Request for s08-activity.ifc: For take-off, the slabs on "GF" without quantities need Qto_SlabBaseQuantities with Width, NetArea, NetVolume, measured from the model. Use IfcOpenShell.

First a look at what the model holds.

```python
import ifcopenshell
import ifcopenshell.util.element
import ifcopenshell.util.unit

model = ifcopenshell.open("s08-activity.ifc")
print(model.schema)
for unit_type in ("LENGTHUNIT", "AREAUNIT", "VOLUMEUNIT"):
    print(unit_type, ifcopenshell.util.unit.calculate_unit_scale(model, unit_type))
storey = next(s for s in model.by_type("IfcBuildingStorey") if s.Name == "GF")
slabs = [e for e in ifcopenshell.util.element.get_decomposition(storey) if e.is_a("IfcSlab")]
for e in sorted(slabs, key=lambda e: e.id()):
    print(e.id(), e.is_a(), e.Name, list(ifcopenshell.util.element.get_psets(e, qtos_only=True)), sep=" | ")
```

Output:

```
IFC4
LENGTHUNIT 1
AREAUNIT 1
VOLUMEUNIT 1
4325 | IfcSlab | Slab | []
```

```python
import ifcopenshell
import ifcopenshell.api.pset
import ifcopenshell.geom
import ifcopenshell.util.element
import ifcopenshell.util.shape
import ifcopenshell.util.unit

model = ifcopenshell.open("s08-activity.ifc")
unit_scale = ifcopenshell.util.unit.calculate_unit_scale(model)
area_scale = ifcopenshell.util.unit.calculate_unit_scale(model, "AREAUNIT")
volume_scale = ifcopenshell.util.unit.calculate_unit_scale(model, "VOLUMEUNIT")
settings = ifcopenshell.geom.settings()

storey = next(s for s in model.by_type("IfcBuildingStorey") if s.Name == "GF")
slabs = [e for e in ifcopenshell.util.element.get_decomposition(storey) if e.is_a("IfcSlab")]

for e in sorted(slabs, key=lambda e: e.id()):
    if ifcopenshell.util.element.get_psets(e, qtos_only=True, should_inherit=False):
        continue
    # Geometry comes back in metres, in the element's own axes.
    shape = ifcopenshell.geom.create_shape(settings, e)
    values = {
        "Width": ifcopenshell.util.shape.get_z(shape.geometry) / unit_scale,
        "NetArea": ifcopenshell.util.shape.get_footprint_area(shape.geometry) / area_scale,
        "NetVolume": ifcopenshell.util.shape.get_volume(shape.geometry) / volume_scale,
    }
    qto = ifcopenshell.api.pset.add_qto(model, product=e, name="Qto_SlabBaseQuantities")
    ifcopenshell.api.pset.edit_qto(model, qto=qto, properties=values)
    print(e.id(), {k: round(v, 3) for k, v in values.items()})

model.write("s08-activity_updated.ifc")
```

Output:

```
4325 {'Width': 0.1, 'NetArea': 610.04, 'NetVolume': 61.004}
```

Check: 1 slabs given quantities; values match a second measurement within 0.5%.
